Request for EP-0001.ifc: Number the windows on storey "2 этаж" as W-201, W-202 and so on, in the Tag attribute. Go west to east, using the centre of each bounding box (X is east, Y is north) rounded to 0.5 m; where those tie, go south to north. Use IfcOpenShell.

First a look at what the model holds.

```python
import ifcopenshell
import ifcopenshell.util.element
import ifcopenshell.util.placement

model = ifcopenshell.open("EP-0001.ifc")
print(model.schema)
storey = next(s for s in model.by_type("IfcBuildingStorey") if s.Name == "2 этаж")
windows = [e for e in ifcopenshell.util.element.get_decomposition(storey) if e.is_a("IfcWindow")]
for e in sorted(windows, key=lambda e: e.id()):
    origin = ifcopenshell.util.placement.get_local_placement(e.ObjectPlacement)[:3, 3]
    print(e.id(), e.Tag, e.Name, origin.round(2) + 0.0, sep=" | ")
```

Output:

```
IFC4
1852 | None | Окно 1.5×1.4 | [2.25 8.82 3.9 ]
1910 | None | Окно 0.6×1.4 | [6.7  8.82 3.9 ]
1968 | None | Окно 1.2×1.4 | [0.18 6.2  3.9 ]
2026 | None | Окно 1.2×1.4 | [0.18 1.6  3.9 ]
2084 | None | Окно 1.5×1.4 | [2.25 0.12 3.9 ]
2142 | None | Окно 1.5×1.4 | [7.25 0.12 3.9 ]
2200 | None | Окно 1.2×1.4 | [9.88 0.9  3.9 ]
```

```python
import ifcopenshell
import ifcopenshell.geom
import ifcopenshell.util.element
import ifcopenshell.util.shape

model = ifcopenshell.open("EP-0001.ifc")
settings = ifcopenshell.geom.settings()
settings.set("use-world-coords", True)


def centre(element):
    shape = ifcopenshell.geom.create_shape(settings, element)
    return ifcopenshell.util.shape.get_bbox_centroid(shape.geometry)


storey = next(s for s in model.by_type("IfcBuildingStorey") if s.Name == "2 этаж")
windows = [e for e in ifcopenshell.util.element.get_decomposition(storey) if e.is_a("IfcWindow")]

# Insertion points can sit at a corner or the storey origin, so sort by the geometry (in metres).
centres = {e: centre(e) for e in windows}
windows.sort(key=lambda e: (round(centres[e][0] / 0.5), centres[e][1]))

for i, e in enumerate(windows, start=1):
    number = f"W-2{i:02d}"
    e.Tag = number
    print(e.id(), number)

model.write("EP-0001_updated.ifc")
```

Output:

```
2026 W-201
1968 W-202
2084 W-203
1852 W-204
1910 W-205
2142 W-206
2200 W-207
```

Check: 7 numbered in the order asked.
